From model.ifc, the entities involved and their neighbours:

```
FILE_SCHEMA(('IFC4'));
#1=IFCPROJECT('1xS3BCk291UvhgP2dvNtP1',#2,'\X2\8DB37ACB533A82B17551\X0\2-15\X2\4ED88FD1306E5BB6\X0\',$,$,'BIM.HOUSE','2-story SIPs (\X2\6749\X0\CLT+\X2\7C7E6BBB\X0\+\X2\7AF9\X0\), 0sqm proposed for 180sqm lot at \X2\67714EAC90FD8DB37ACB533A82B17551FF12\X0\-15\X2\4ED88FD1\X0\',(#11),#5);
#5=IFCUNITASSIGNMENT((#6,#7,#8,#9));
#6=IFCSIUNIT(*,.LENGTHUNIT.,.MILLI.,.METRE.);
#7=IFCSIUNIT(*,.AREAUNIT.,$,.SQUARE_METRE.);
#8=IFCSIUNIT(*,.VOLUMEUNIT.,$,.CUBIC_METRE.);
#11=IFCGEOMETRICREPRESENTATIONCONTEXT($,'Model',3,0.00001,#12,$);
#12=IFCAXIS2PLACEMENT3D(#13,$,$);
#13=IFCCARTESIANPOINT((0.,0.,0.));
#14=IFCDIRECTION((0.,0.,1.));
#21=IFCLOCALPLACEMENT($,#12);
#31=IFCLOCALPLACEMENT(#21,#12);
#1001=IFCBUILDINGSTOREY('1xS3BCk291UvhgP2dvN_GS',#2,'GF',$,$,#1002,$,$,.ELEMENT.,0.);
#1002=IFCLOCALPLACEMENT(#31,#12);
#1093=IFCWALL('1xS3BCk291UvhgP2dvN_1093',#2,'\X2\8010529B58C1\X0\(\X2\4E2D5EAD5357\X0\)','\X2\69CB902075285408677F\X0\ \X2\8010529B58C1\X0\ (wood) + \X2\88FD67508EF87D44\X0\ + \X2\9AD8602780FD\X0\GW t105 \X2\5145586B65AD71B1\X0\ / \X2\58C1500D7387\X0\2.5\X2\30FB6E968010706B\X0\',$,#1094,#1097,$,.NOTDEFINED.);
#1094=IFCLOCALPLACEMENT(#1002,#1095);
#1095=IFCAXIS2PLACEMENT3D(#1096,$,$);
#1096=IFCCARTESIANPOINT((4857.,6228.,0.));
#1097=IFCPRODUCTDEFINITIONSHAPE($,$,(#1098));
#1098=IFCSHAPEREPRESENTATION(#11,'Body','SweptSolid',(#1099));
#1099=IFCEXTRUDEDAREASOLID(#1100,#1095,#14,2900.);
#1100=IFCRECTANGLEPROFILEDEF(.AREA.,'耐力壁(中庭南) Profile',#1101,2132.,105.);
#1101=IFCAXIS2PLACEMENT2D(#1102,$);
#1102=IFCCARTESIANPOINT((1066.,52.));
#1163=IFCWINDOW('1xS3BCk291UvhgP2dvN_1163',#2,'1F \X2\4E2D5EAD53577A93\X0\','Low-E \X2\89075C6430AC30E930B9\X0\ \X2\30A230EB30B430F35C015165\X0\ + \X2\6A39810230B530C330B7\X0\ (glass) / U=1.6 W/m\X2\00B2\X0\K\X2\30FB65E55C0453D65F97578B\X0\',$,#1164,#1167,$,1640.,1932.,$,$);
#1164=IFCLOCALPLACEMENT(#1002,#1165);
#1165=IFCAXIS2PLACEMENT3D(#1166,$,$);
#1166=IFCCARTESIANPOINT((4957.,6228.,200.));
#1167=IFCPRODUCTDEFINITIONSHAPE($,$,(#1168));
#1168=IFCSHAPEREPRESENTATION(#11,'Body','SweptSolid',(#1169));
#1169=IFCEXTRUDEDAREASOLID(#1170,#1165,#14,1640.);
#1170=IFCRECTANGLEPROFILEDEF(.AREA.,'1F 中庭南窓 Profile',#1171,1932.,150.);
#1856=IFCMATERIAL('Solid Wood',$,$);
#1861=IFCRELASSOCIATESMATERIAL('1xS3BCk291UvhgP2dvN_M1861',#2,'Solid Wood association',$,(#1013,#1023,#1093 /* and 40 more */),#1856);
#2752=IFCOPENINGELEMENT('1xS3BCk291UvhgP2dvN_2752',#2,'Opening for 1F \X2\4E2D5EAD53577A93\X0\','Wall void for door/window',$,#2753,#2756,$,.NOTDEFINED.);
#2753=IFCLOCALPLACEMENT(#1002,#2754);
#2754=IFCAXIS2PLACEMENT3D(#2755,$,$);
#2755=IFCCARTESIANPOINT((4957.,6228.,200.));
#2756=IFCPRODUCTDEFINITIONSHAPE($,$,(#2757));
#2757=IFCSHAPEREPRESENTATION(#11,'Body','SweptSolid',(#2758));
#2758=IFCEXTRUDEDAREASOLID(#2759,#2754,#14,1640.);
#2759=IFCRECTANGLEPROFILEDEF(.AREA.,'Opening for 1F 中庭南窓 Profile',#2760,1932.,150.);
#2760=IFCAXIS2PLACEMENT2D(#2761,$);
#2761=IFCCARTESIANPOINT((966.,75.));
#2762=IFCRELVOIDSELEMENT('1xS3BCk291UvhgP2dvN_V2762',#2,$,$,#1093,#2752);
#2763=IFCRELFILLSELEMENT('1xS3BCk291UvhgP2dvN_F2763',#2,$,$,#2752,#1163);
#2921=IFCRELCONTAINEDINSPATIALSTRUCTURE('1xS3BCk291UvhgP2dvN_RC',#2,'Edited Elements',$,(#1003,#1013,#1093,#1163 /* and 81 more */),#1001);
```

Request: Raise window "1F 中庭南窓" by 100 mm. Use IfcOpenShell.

```python
import numpy as np
import ifcopenshell
import ifcopenshell.api.geometry
import ifcopenshell.util.placement
import ifcopenshell.util.unit

model = ifcopenshell.open("model.ifc")
unit_scale = ifcopenshell.util.unit.calculate_unit_scale(model)

window = model.by_guid("1xS3BCk291UvhgP2dvN_1163")
opening = window.FillsVoids[0].RelatingOpeningElement
dz = 100.0

shift = np.array([0.0, 0.0, dz])
# The window is not placed relative to its opening, so move both.
for product in (opening, window):
    matrix = ifcopenshell.util.placement.get_local_placement(product.ObjectPlacement)
    matrix[:3, 3] += shift
    ifcopenshell.api.geometry.edit_object_placement(model, product=product, matrix=matrix, is_si=False)

print(f"moved by {dz * unit_scale:+.3f} m")

model.write("model-out.ifc")
```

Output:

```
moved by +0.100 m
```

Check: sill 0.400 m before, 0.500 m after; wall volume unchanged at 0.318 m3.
